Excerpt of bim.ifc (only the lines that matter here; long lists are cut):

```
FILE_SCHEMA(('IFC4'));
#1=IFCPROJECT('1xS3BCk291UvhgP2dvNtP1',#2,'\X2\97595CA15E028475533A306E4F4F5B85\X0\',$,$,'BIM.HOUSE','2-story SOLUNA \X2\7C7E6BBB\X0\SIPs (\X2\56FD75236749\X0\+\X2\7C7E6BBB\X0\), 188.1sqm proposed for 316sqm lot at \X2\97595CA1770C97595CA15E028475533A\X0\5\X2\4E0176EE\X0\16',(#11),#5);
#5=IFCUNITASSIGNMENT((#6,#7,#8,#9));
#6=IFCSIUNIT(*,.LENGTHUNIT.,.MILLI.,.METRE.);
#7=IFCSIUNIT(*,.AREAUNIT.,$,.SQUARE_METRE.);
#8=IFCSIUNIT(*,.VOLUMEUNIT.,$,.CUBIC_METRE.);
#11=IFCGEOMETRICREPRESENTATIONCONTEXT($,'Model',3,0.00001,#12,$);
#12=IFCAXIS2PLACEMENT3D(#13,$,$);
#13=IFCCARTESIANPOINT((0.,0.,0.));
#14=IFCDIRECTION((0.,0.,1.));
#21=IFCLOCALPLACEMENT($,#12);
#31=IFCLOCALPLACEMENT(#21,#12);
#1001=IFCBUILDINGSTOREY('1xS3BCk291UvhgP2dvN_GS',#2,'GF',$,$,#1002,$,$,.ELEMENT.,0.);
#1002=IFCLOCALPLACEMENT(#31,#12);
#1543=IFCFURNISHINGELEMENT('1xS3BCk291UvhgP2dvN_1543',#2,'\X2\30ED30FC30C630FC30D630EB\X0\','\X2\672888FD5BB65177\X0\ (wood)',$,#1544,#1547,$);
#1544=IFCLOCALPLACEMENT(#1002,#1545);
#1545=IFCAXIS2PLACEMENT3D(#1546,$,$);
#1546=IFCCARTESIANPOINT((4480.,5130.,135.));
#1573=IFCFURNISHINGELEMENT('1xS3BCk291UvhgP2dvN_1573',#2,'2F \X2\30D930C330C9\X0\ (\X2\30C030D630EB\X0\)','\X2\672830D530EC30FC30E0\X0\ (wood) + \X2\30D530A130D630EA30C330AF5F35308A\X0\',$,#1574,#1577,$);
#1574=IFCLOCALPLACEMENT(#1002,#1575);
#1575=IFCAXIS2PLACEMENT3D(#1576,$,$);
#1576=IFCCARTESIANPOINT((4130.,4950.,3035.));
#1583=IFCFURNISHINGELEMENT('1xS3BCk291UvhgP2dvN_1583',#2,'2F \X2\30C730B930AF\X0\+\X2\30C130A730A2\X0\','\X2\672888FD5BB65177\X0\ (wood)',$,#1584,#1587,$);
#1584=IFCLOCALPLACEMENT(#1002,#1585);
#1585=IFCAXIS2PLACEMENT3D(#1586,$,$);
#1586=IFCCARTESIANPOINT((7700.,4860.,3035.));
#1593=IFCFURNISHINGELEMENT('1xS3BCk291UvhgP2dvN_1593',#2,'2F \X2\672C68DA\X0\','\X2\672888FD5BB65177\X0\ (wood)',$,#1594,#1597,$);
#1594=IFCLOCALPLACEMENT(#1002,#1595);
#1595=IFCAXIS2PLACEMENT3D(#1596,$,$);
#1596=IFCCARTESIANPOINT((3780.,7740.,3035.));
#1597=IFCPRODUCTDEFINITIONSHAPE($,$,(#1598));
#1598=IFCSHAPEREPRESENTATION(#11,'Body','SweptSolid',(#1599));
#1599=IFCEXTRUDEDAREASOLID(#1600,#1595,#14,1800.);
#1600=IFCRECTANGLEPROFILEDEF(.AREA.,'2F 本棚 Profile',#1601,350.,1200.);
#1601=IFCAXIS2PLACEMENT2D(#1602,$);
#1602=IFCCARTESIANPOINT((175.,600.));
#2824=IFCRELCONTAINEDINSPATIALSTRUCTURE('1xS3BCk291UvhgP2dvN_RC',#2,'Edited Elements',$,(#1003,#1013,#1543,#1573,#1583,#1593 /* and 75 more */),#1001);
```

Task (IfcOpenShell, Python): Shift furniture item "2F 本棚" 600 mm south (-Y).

```python
import ifcopenshell
import ifcopenshell.api.geometry
import ifcopenshell.util.placement
import ifcopenshell.util.unit

model = ifcopenshell.open("bim.ifc")
unit_scale = ifcopenshell.util.unit.calculate_unit_scale(model)

item = model.by_guid("1xS3BCk291UvhgP2dvN_1593")
matrix = ifcopenshell.util.placement.get_local_placement(item.ObjectPlacement)
matrix[1, 3] -= 0.6 / unit_scale
ifcopenshell.api.geometry.edit_object_placement(model, product=item, matrix=matrix, is_si=False)

print(ifcopenshell.util.placement.get_local_placement(item.ObjectPlacement).round(3) + 0.0)

model.write("bim_rev.ifc")
```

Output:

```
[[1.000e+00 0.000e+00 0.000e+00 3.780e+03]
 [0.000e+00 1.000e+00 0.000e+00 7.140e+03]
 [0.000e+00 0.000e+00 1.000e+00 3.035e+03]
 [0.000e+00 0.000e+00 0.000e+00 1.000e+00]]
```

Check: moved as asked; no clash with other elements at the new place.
